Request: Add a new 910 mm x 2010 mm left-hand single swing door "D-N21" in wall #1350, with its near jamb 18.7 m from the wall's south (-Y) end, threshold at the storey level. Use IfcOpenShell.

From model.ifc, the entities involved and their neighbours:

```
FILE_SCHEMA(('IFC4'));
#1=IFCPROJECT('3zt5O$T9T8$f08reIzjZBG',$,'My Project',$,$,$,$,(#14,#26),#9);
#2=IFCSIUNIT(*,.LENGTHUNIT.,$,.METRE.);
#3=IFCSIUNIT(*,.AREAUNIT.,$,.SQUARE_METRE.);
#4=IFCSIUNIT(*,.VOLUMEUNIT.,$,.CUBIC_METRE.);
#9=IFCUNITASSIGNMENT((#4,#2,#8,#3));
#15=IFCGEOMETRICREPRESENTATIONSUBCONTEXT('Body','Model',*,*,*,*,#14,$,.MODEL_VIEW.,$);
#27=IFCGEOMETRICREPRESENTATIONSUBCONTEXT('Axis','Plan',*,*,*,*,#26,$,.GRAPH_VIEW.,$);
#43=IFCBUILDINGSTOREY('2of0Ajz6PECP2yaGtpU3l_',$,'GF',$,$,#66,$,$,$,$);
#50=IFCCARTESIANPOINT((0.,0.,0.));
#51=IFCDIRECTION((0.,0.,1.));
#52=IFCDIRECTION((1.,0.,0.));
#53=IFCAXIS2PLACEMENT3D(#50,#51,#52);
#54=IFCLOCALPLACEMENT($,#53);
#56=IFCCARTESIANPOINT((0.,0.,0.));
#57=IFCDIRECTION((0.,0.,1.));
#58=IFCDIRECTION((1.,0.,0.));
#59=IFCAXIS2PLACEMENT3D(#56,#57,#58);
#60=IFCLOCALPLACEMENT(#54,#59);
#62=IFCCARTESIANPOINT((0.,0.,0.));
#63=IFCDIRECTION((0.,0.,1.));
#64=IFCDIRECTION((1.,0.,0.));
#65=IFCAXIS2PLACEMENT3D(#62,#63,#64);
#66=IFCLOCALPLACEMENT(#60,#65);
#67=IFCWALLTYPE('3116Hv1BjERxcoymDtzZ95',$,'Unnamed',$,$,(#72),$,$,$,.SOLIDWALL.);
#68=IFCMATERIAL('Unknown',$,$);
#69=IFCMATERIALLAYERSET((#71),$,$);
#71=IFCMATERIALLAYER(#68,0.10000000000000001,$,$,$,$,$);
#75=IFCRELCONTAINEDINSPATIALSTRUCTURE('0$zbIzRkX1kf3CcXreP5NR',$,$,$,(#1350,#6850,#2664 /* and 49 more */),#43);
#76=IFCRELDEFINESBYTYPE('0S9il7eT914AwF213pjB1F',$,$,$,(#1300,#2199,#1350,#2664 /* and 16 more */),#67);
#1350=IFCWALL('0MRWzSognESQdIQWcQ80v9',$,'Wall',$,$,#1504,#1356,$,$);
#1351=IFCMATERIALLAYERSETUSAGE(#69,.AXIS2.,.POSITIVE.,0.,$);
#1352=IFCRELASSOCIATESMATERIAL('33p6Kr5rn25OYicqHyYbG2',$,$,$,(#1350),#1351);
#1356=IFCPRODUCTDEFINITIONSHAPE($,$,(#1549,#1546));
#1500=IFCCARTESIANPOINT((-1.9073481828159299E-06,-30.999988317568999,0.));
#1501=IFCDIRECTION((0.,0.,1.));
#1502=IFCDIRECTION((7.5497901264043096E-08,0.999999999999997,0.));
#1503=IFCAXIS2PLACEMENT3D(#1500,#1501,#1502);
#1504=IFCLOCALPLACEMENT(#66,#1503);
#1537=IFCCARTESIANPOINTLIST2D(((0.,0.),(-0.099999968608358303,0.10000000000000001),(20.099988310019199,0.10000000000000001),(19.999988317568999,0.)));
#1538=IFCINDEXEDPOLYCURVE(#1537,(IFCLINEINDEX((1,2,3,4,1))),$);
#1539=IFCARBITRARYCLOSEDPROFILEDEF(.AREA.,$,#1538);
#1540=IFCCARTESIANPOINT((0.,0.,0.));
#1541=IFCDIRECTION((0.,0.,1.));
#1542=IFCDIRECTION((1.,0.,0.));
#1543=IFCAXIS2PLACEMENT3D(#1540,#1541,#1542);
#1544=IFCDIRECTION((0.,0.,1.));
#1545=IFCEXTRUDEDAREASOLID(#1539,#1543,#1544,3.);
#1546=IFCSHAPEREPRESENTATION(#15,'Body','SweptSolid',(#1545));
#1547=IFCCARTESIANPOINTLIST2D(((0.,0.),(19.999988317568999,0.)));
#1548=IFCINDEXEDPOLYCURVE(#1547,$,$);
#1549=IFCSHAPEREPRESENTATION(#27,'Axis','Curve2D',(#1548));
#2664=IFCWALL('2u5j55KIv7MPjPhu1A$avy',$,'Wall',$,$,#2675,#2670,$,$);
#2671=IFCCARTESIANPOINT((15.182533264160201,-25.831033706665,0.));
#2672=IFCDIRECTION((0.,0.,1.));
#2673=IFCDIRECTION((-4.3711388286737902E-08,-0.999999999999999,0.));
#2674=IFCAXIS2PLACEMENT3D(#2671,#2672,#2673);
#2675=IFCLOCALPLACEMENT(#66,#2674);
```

```python
import numpy as np
import ifcopenshell
import ifcopenshell.api.feature
import ifcopenshell.api.geometry
import ifcopenshell.api.root
import ifcopenshell.api.spatial
import ifcopenshell.geom
import ifcopenshell.util.element
import ifcopenshell.util.placement
import ifcopenshell.util.representation
import ifcopenshell.util.shape
import ifcopenshell.util.unit

model = ifcopenshell.open("model.ifc")
unit_scale = ifcopenshell.util.unit.calculate_unit_scale(model)
settings = ifcopenshell.geom.settings()


def volume(element):
    """Net volume in cubic metres, openings subtracted."""
    shape = ifcopenshell.geom.create_shape(settings, element)
    return ifcopenshell.util.shape.get_volume(shape.geometry)


wall = model.by_id(1350)
storey = ifcopenshell.util.element.get_container(wall, ifc_class="IfcBuildingStorey")
context = ifcopenshell.util.representation.get_context(model, "Model", "Body", "MODEL_VIEW")
before = volume(wall)

width, height, from_end, sill = 0.91, 2.01, 18.7, 0.0  # metres

# The wall runs along its own X axis, and the end named is its -X end.
wall_shape = ifcopenshell.geom.create_shape(settings, wall)
x, y, z = ifcopenshell.util.shape.get_vertices(wall_shape.geometry).T
start = x.min() + from_end
face, thickness = float(y.min()), float(y.max() - y.min())
wall_matrix = ifcopenshell.util.placement.get_local_placement(wall.ObjectPlacement)
level = ifcopenshell.util.placement.get_local_placement(storey.ObjectPlacement)[2, 3]


def in_wall(x, y):
    """Placement at x, y metres in the wall's axes, at sill height."""
    matrix = wall_matrix.copy()
    matrix[:, 3] = wall_matrix @ np.array([x / unit_scale, y / unit_scale, 0.0, 1.0])
    matrix[2, 3] = level + sill / unit_scale
    return matrix


# Opening: a box that overshoots both wall faces by 50 mm.
opening = ifcopenshell.api.root.create_entity(model, ifc_class="IfcOpeningElement", predefined_type="OPENING")
box = ifcopenshell.api.geometry.add_wall_representation(
    model, context=context, length=width, height=height, thickness=thickness + 0.1
)
ifcopenshell.api.geometry.assign_representation(model, product=opening, representation=box)
ifcopenshell.api.geometry.edit_object_placement(model, product=opening, matrix=in_wall(start, face - 0.05), is_si=False)
ifcopenshell.api.feature.add_feature(model, feature=opening, element=wall)

door = ifcopenshell.api.root.create_entity(model, ifc_class="IfcDoor", name="D-N21", predefined_type="DOOR")
door.OverallWidth, door.OverallHeight = width / unit_scale, height / unit_scale
door.OperationType = "SINGLE_SWING_LEFT"
body = ifcopenshell.api.geometry.add_door_representation(
    model,
    context=context,
    overall_width=door.OverallWidth,
    overall_height=door.OverallHeight,
    operation_type="SINGLE_SWING_LEFT",
    lining_properties={"LiningDepth": thickness / unit_scale, "ThresholdDepth": thickness / unit_scale},
)
ifcopenshell.api.geometry.assign_representation(model, product=door, representation=body)
ifcopenshell.api.spatial.assign_container(model, products=[door], relating_structure=storey)
ifcopenshell.api.feature.add_filling(model, opening=opening, element=door)

# The lining spans the wall, so the door starts at the wall face.
ifcopenshell.api.geometry.edit_object_placement(model, product=door, matrix=in_wall(start, face), is_si=False)

after = volume(wall)

print(f"wall volume {before:.3f} -> {after:.3f} m3")

model.write("model_updated.ifc")
```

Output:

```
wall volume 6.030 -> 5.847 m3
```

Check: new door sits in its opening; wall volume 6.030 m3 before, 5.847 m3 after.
